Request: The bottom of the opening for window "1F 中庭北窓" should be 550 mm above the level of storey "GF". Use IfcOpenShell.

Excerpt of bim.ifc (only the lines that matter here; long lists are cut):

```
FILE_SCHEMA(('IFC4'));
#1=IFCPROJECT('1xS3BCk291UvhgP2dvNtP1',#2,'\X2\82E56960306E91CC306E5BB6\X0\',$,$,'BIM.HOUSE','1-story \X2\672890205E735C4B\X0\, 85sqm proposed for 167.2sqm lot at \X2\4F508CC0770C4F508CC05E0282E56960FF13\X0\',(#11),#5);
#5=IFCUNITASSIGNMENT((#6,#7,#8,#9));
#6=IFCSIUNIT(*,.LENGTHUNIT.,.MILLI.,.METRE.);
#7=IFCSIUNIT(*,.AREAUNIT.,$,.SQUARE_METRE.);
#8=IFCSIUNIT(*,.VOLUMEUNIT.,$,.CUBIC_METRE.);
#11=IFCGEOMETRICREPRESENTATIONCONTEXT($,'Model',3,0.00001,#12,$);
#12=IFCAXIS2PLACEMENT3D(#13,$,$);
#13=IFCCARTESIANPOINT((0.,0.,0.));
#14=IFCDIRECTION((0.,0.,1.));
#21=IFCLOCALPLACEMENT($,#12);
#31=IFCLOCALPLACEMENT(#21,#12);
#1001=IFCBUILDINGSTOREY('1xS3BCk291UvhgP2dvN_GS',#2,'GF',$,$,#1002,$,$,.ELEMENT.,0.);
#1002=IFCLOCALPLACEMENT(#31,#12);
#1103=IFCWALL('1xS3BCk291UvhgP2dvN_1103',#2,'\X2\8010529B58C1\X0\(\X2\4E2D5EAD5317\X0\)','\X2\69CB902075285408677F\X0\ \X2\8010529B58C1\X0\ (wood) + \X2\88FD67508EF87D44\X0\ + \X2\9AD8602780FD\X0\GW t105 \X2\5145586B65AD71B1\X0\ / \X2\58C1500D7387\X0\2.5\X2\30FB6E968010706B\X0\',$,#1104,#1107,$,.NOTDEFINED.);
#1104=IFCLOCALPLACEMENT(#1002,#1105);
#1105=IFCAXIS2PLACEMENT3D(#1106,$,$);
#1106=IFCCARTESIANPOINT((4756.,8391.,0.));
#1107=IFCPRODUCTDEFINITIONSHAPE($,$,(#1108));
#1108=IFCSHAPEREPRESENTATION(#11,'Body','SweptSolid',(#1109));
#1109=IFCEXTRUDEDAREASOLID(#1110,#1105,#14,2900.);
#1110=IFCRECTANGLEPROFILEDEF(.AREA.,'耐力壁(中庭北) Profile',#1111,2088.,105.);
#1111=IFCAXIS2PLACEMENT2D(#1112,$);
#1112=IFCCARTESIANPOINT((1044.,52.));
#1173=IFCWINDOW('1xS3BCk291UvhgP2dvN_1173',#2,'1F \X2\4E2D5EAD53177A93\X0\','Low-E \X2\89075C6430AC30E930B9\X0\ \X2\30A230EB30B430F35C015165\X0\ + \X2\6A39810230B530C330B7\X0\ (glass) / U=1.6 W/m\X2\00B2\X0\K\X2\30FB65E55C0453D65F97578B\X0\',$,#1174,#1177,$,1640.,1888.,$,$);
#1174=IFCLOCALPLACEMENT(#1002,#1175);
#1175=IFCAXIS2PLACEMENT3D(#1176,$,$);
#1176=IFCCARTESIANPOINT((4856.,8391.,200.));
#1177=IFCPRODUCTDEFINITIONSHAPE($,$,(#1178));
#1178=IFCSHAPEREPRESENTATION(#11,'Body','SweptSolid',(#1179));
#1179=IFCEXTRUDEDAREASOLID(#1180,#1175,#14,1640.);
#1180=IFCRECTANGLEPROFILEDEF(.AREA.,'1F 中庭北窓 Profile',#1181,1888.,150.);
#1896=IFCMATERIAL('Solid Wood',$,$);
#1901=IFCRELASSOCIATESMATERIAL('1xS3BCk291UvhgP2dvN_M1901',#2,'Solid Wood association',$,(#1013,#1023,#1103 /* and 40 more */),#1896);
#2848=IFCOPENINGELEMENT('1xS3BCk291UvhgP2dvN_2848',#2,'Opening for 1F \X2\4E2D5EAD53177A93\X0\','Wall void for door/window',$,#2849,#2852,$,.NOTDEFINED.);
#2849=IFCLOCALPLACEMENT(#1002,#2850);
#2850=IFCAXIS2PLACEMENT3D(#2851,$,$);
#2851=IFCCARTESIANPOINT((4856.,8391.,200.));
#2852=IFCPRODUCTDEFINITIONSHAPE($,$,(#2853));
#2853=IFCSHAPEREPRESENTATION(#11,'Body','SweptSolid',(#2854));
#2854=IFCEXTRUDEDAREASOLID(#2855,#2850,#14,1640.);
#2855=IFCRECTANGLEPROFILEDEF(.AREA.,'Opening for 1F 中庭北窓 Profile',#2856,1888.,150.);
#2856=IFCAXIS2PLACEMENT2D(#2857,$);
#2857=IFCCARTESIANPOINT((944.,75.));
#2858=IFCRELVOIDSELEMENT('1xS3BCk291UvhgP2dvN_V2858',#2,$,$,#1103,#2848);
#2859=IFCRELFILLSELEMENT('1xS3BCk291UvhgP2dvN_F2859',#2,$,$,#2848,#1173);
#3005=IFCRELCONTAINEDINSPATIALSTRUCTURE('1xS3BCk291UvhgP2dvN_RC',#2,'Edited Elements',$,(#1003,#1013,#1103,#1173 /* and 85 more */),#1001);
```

```python
import numpy as np
import ifcopenshell
import ifcopenshell.api.geometry
import ifcopenshell.geom
import ifcopenshell.util.element
import ifcopenshell.util.placement
import ifcopenshell.util.shape
import ifcopenshell.util.unit

model = ifcopenshell.open("bim.ifc")
unit_scale = ifcopenshell.util.unit.calculate_unit_scale(model)

window = model.by_id(1173)
opening = window.FillsVoids[0].RelatingOpeningElement
storey = ifcopenshell.util.element.get_container(window, ifc_class="IfcBuildingStorey")
level = ifcopenshell.util.placement.get_local_placement(storey.ObjectPlacement)[2, 3]

# The opening's origin need not be at the sill, so measure its lowest point.
shape = ifcopenshell.geom.create_shape(ifcopenshell.geom.settings(), opening)
bottom = ifcopenshell.util.shape.get_shape_bottom_elevation(shape, shape.geometry) / unit_scale
dz = level + 550.0 - bottom

shift = np.array([0.0, 0.0, dz])
# The window is not placed relative to its opening, so move both.
for product in (opening, window):
    matrix = ifcopenshell.util.placement.get_local_placement(product.ObjectPlacement)
    matrix[:3, 3] += shift
    ifcopenshell.api.geometry.edit_object_placement(model, product=product, matrix=matrix, is_si=False)

print(f"moved by {dz * unit_scale:+.3f} m")

model.write("bim-out.ifc")
```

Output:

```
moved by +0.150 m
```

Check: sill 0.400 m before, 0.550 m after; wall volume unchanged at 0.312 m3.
